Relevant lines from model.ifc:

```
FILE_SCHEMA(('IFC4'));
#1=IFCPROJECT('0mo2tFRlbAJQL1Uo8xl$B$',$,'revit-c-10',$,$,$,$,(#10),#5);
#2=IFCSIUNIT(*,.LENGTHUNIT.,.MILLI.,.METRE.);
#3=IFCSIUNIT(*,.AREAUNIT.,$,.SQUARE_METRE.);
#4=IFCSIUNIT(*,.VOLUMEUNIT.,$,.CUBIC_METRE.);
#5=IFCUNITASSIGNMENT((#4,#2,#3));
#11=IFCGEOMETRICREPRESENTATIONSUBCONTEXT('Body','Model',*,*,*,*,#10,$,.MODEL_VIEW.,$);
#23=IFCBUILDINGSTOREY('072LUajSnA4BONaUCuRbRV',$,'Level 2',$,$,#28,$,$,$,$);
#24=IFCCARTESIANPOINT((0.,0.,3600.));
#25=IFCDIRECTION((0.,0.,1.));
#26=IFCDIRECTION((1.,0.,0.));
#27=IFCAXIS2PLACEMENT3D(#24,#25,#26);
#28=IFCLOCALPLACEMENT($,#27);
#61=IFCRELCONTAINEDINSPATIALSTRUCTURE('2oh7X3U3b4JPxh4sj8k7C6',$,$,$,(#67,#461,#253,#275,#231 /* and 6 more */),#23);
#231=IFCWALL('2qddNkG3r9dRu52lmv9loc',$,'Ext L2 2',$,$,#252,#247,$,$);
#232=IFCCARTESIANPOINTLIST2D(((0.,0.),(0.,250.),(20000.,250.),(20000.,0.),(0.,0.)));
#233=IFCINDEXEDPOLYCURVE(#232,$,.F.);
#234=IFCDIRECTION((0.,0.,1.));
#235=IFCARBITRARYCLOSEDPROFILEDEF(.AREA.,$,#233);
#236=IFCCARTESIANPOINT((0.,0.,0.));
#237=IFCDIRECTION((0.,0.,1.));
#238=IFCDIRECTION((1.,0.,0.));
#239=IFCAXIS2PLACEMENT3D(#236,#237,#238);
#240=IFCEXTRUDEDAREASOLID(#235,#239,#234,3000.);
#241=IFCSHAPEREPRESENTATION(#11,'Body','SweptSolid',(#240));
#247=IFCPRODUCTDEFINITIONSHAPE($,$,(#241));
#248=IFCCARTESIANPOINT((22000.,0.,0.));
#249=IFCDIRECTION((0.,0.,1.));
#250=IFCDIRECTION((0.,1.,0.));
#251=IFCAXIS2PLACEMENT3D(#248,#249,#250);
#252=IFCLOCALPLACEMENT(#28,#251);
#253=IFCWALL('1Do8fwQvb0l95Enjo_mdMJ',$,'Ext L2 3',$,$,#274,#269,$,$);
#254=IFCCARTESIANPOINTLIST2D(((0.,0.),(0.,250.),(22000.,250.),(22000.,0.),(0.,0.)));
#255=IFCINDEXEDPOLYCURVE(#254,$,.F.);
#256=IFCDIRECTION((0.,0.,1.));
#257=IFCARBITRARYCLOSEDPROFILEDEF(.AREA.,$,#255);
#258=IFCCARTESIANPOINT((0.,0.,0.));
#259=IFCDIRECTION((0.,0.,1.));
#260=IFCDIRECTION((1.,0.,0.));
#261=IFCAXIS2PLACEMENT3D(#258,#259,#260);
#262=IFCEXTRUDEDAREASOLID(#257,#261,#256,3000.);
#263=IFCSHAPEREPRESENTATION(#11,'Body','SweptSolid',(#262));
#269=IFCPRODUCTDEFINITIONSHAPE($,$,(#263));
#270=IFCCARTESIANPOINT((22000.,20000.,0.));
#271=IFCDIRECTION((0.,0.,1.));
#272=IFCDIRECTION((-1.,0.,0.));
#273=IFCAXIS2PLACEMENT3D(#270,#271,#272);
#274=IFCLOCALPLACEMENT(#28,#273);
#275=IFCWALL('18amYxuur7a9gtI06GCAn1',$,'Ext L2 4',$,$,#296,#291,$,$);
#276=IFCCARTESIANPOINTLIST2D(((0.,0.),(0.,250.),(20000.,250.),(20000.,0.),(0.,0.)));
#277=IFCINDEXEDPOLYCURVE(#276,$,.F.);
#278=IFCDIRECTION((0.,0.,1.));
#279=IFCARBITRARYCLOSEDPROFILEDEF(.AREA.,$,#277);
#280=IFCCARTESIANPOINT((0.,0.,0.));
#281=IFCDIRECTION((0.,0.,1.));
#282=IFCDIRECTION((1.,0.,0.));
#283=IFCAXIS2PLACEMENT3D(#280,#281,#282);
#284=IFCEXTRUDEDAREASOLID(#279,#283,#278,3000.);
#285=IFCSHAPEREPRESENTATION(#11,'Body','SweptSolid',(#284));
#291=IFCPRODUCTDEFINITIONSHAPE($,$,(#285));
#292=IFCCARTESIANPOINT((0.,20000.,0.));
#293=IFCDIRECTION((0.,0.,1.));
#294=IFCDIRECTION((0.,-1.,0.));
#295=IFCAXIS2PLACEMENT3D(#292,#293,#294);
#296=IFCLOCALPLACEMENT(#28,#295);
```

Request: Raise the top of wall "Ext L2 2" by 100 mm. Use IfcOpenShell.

```python
import ifcopenshell
import ifcopenshell.geom
import ifcopenshell.util.representation
import ifcopenshell.util.shape
import ifcopenshell.util.unit

model = ifcopenshell.open("model.ifc")
unit_scale = ifcopenshell.util.unit.calculate_unit_scale(model)
settings = ifcopenshell.geom.settings()


def volume(element):
    """Net volume in cubic metres, openings subtracted."""
    shape = ifcopenshell.geom.create_shape(settings, element)
    return ifcopenshell.util.shape.get_volume(shape.geometry)


wall = model.by_guid("2qddNkG3r9dRu52lmv9loc")
before = volume(wall)

body = ifcopenshell.util.representation.get_representation(wall, "Model", "Body")
solid = body.Items[0]
old_height = solid.Depth
solid.Depth += 0.1 / unit_scale
after = volume(wall)

print(f"height {old_height:g} -> {solid.Depth:g}, volume {before:.3f} -> {after:.3f} m3")

model.write("model_v2.ifc")
```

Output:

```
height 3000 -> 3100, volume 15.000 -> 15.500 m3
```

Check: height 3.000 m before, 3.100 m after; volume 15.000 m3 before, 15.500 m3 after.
